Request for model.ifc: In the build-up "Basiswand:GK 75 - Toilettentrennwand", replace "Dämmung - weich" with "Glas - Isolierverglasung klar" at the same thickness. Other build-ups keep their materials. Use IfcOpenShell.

First a look at what the model holds.

```python
import ifcopenshell
import ifcopenshell.util.element

model = ifcopenshell.open("model.ifc")
print(model.schema)
for layer_set in model.by_type("IfcMaterialLayerSet"):
    if layer_set.LayerSetName == "Basiswand:GK 75 - Toilettentrennwand":
        for layer in layer_set.MaterialLayers:
            print(layer.id(), layer.Material and layer.Material.Name, layer.LayerThickness, sep=" | ")
        print(len(ifcopenshell.util.element.get_elements_by_material(model, layer_set)), "elements and types use it")
print(sorted(m.Name for m in model.by_type("IfcMaterial") if m.Name)[:60])
```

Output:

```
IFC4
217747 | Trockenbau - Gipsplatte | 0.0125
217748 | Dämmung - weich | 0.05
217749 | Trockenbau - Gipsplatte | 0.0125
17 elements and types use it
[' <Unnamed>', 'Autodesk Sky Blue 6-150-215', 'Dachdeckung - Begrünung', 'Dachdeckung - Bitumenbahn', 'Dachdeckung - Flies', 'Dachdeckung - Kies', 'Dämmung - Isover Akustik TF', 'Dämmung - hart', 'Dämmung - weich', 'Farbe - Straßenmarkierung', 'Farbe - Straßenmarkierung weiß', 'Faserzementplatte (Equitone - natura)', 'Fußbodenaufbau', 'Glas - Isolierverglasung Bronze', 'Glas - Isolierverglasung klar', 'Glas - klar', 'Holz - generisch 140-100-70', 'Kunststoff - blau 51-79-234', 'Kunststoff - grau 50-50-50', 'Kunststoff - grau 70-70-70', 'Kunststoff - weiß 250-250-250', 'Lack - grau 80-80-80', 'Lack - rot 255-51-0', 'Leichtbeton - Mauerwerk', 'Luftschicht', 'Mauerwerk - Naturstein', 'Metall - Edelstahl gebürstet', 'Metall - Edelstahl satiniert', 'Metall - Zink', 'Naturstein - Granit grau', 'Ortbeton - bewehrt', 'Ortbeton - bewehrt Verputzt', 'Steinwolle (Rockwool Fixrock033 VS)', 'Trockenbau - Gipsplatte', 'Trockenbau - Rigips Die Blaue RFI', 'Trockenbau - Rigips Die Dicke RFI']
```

```python
import ifcopenshell
import ifcopenshell.api.material

model = ifcopenshell.open("model.ifc")

layer_set = next(s for s in model.by_type("IfcMaterialLayerSet") if s.LayerSetName == "Basiswand:GK 75 - Toilettentrennwand")
layer = next(l for l in layer_set.MaterialLayers if l.Material and l.Material.Name == "Dämmung - weich")
material = next(m for m in model.by_type("IfcMaterial") if m.Name == "Glas - Isolierverglasung klar")

# Point this one layer at the other material; renaming the old one would change it everywhere.
ifcopenshell.api.material.edit_layer(model, layer=layer, attributes={"Name": material.Name}, material=material)

print([l.Material.Name if l.Material else None for l in layer_set.MaterialLayers])

model.write("model_v2.ifc")
```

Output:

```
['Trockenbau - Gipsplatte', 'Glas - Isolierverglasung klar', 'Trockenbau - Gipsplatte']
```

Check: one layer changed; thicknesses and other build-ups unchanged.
